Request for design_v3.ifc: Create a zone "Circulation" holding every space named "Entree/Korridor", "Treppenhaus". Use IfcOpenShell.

First a look at what the model holds.

```python
import ifcopenshell

model = ifcopenshell.open("design_v3.ifc")
print(model.schema)
seen = {}
for space in model.by_type("IfcSpace"):
    seen[space.LongName] = seen.get(space.LongName, 0) + 1
for name, count in sorted(seen.items(), key=str):
    print(count, "x", name)
print("zones:", [z.Name for z in model.by_type("IfcZone")][:20])
```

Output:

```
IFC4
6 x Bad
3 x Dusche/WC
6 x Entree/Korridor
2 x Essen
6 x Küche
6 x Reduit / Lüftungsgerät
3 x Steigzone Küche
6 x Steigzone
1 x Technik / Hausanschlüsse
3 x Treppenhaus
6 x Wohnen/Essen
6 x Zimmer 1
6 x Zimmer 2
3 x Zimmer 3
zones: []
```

```python
import ifcopenshell
import ifcopenshell.api.group
import ifcopenshell.api.root

model = ifcopenshell.open("design_v3.ifc")

names = {"Entree/Korridor", "Treppenhaus"}
spaces = [s for s in model.by_type("IfcSpace") if s.LongName in names]

zone = ifcopenshell.api.root.create_entity(model, ifc_class="IfcZone", name="Circulation")
ifcopenshell.api.group.assign_group(model, products=spaces, group=zone)
print(len(spaces), "spaces in", zone.Name)

model.write("design_v3_v2.ifc")
```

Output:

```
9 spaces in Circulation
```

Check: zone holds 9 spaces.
